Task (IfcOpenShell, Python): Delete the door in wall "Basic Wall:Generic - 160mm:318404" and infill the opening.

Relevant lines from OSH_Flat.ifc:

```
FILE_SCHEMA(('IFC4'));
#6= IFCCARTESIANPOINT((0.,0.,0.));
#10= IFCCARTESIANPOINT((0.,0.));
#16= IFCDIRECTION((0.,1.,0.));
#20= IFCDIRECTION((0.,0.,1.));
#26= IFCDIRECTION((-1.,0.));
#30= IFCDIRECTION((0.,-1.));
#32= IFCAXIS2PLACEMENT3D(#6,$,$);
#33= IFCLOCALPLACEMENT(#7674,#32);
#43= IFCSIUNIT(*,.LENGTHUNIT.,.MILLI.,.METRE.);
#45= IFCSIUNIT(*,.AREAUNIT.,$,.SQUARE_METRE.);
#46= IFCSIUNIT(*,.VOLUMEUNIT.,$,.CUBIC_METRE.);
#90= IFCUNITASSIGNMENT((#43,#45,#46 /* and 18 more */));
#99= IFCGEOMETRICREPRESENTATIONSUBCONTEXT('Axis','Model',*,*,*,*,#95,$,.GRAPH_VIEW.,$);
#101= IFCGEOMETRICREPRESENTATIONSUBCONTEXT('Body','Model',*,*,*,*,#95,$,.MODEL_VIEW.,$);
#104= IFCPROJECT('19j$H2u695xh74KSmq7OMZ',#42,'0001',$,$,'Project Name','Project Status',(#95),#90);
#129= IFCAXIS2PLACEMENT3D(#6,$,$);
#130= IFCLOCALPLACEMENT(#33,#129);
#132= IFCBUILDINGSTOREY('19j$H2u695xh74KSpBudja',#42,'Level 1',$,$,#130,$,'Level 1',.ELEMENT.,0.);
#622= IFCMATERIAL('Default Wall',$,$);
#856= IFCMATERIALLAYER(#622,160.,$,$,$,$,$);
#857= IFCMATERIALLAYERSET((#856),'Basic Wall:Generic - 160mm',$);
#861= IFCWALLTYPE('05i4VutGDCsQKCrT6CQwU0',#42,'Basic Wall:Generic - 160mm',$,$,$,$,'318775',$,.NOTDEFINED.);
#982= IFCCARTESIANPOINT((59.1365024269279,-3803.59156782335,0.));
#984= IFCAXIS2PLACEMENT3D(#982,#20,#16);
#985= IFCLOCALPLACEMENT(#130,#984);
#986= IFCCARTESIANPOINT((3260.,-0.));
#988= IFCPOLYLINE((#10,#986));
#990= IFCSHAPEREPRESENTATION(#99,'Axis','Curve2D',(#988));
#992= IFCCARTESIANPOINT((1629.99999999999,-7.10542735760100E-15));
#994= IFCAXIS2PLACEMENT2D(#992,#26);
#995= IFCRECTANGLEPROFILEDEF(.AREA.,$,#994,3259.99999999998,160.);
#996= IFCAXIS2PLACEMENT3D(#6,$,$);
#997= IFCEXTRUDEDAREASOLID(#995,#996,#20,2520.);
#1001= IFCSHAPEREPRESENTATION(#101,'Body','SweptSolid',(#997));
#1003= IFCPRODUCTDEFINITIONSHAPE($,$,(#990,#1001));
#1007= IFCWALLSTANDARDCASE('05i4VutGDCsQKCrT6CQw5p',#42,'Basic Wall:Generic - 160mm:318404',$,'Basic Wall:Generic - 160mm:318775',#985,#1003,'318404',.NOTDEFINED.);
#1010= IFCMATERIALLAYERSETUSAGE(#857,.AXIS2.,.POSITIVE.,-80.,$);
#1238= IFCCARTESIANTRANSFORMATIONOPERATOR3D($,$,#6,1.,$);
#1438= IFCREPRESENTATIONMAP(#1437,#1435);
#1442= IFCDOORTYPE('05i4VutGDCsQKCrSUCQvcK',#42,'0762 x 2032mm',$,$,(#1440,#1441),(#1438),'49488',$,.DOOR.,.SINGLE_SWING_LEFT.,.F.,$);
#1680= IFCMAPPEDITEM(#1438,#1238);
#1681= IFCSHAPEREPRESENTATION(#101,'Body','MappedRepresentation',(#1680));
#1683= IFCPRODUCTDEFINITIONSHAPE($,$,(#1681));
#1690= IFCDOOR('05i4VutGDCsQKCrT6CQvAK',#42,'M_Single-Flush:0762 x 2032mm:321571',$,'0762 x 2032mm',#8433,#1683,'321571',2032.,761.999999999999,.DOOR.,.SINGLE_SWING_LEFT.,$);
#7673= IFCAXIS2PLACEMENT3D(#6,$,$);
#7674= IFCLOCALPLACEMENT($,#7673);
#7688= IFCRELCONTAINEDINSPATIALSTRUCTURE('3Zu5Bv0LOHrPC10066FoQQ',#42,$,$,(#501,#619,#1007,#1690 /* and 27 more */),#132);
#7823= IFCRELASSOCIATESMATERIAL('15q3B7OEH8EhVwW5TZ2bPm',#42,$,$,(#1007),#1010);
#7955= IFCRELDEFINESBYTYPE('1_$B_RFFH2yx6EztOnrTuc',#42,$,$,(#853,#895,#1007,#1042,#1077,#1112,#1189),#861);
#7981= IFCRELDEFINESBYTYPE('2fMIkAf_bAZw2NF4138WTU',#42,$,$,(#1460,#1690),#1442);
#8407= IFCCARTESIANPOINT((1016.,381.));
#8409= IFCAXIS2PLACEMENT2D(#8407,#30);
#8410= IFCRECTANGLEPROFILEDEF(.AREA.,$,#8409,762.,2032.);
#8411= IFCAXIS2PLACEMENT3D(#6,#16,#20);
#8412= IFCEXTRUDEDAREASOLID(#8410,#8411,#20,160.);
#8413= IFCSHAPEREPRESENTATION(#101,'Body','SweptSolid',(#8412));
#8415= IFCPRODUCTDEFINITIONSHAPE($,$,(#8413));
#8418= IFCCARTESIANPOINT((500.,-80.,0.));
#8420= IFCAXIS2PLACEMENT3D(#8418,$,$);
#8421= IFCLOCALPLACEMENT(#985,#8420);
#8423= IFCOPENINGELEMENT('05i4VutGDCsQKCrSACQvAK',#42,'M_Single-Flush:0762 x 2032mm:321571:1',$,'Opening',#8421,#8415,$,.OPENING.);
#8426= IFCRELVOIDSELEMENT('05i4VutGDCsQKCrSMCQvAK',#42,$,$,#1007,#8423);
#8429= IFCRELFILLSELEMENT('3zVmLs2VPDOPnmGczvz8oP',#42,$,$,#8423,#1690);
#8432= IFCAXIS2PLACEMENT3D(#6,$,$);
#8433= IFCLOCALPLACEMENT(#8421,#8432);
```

```python
import ifcopenshell
import ifcopenshell.api.feature
import ifcopenshell.api.root
import ifcopenshell.geom
import ifcopenshell.util.shape

model = ifcopenshell.open("OSH_Flat.ifc")
settings = ifcopenshell.geom.settings()


def volume(element):
    """Net volume in cubic metres, openings subtracted."""
    shape = ifcopenshell.geom.create_shape(settings, element)
    return ifcopenshell.util.shape.get_volume(shape.geometry)


door = model.by_guid("05i4VutGDCsQKCrT6CQvAK")
opening = door.FillsVoids[0].RelatingOpeningElement
wall = opening.VoidsElements[0].RelatingBuildingElement
before = volume(wall)

ifcopenshell.api.root.remove_product(model, product=door)
ifcopenshell.api.feature.remove_feature(model, feature=opening)

after = volume(wall)

print(f"wall volume {before:.3f} -> {after:.3f} m3")

model.write("OSH_Flat_rev.ifc")
```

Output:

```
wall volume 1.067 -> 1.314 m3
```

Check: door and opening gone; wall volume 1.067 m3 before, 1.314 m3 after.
